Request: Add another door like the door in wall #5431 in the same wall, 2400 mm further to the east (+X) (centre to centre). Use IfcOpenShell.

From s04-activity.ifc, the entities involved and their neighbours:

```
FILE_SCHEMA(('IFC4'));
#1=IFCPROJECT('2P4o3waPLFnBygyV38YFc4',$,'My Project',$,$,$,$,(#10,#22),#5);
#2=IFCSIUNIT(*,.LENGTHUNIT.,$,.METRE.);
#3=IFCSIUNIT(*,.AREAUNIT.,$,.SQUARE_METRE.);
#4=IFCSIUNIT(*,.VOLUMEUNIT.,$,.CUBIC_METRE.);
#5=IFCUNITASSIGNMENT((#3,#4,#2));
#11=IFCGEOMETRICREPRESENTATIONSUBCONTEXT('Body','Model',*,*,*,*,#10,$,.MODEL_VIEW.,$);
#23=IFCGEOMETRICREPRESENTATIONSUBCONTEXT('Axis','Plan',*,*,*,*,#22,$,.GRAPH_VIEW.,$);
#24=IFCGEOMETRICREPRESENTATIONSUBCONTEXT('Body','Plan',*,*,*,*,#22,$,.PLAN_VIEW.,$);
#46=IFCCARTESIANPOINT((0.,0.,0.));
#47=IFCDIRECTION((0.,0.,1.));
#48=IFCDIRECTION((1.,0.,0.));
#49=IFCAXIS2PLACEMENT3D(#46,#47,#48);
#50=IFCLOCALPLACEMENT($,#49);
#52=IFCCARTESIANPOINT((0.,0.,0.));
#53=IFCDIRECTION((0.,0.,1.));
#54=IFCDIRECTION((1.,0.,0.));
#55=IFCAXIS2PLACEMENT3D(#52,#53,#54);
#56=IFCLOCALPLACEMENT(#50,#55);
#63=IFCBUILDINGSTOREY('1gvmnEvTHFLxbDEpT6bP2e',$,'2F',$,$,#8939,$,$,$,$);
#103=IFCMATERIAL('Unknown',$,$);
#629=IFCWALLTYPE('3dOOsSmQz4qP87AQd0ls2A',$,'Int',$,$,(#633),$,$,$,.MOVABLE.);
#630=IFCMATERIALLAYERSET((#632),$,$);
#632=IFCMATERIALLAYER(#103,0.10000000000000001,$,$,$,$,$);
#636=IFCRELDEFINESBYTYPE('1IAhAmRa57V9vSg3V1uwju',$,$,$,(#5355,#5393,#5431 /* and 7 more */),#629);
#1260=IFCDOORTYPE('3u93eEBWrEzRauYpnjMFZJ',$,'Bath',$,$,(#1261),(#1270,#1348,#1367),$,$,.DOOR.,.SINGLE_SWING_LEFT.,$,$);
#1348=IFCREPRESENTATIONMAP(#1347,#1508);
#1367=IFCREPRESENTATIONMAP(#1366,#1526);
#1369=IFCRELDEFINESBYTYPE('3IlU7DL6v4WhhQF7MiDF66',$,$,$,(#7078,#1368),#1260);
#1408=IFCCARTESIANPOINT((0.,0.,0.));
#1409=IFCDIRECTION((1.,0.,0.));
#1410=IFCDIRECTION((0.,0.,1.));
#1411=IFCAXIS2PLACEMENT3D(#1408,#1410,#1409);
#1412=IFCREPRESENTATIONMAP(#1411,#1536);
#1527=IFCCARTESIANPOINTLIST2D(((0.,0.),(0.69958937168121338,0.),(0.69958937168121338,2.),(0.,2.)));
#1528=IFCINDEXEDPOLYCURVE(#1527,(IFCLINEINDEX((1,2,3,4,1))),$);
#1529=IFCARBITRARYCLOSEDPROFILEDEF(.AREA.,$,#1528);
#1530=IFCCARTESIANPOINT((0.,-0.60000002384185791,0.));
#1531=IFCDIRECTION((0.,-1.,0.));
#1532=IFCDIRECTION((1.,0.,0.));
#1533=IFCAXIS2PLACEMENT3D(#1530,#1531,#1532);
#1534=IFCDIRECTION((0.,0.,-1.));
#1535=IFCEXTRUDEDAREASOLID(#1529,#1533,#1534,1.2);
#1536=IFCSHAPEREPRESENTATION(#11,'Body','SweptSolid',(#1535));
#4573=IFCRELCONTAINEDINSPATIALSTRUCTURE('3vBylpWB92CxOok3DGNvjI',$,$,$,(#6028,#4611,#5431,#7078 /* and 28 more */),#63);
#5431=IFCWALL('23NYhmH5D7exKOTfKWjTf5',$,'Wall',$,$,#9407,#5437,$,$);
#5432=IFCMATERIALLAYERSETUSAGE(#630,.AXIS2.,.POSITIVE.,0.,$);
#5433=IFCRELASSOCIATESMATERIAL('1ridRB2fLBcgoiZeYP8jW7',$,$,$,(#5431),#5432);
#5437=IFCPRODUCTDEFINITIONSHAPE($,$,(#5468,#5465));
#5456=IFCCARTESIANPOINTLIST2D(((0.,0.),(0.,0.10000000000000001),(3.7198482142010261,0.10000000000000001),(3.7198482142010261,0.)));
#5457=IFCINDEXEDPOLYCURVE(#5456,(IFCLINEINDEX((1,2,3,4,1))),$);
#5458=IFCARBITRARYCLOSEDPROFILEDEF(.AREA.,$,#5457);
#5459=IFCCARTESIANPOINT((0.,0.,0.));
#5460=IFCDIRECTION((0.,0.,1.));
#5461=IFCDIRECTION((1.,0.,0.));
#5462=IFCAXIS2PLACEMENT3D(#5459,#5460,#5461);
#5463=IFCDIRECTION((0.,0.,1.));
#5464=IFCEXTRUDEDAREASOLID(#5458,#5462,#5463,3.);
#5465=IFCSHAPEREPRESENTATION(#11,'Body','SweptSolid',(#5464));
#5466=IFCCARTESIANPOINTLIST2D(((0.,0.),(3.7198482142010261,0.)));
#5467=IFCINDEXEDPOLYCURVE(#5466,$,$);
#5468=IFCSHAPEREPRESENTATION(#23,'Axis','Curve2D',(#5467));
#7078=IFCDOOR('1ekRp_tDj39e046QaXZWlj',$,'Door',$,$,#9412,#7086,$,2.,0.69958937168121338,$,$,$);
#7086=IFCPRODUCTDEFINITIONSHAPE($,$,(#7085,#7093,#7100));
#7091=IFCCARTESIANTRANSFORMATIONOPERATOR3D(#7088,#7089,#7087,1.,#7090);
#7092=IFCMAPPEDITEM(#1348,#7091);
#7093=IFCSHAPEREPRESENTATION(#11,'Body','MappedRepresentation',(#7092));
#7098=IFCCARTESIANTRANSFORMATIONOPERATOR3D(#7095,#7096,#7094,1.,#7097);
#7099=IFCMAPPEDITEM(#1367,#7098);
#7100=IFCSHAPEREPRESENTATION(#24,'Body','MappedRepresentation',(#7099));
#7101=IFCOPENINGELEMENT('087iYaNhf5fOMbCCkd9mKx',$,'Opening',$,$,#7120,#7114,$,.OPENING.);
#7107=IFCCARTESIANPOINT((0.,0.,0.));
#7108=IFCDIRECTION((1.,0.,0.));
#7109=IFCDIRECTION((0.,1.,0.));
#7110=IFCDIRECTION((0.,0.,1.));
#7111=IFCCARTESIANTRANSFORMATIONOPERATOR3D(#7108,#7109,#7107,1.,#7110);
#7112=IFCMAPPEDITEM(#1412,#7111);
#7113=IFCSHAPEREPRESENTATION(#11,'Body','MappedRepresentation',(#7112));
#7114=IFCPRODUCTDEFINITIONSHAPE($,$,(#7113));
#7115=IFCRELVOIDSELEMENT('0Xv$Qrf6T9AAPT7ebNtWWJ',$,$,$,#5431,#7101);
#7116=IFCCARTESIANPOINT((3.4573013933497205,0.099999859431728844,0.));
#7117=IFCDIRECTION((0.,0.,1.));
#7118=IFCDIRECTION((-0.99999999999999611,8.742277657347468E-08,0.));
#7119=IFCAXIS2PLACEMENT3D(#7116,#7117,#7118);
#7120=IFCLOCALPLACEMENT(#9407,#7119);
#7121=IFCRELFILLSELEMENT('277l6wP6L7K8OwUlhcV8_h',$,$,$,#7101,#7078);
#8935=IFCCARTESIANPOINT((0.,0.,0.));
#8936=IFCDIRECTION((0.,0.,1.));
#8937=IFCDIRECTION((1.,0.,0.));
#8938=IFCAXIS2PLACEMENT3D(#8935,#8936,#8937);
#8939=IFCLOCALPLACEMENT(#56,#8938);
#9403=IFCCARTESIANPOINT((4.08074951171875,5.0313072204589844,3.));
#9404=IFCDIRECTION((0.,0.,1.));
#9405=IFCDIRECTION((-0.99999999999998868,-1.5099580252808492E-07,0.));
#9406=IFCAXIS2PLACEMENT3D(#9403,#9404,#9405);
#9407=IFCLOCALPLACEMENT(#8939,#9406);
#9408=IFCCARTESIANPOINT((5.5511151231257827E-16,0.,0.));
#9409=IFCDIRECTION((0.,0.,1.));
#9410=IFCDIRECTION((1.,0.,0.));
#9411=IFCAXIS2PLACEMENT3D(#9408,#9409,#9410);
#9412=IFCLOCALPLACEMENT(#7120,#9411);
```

```python
import ifcopenshell
import ifcopenshell.api.feature
import ifcopenshell.api.geometry
import ifcopenshell.api.root
import ifcopenshell.geom
import ifcopenshell.util.element
import ifcopenshell.util.placement
import ifcopenshell.util.shape

model = ifcopenshell.open("s04-activity.ifc")
settings = ifcopenshell.geom.settings()


def volume(element):
    """Net volume in cubic metres, openings subtracted."""
    shape = ifcopenshell.geom.create_shape(settings, element)
    return ifcopenshell.util.shape.get_volume(shape.geometry)


door = model.by_guid("1ekRp_tDj39e046QaXZWlj")
opening = door.FillsVoids[0].RelatingOpeningElement
wall = opening.VoidsElements[0].RelatingBuildingElement
before = volume(wall)
shift = ifcopenshell.util.placement.get_local_placement(wall.ObjectPlacement)[:3, 0] * -2.4

# copy_class copies the void relationship, type, container and properties, but no geometry.
new_opening = ifcopenshell.api.root.copy_class(model, product=opening)
new_opening.Representation = ifcopenshell.util.element.copy_deep(
    model, opening.Representation, exclude=["IfcGeometricRepresentationContext", "IfcRepresentationMap"]
)
new_door = ifcopenshell.api.root.copy_class(model, product=door)
new_door.Representation = ifcopenshell.util.element.copy_deep(
    model, door.Representation, exclude=["IfcGeometricRepresentationContext", "IfcRepresentationMap"]
)
ifcopenshell.api.feature.add_filling(model, opening=new_opening, element=new_door)

for old, new in ((opening, new_opening), (door, new_door)):
    matrix = ifcopenshell.util.placement.get_local_placement(old.ObjectPlacement)
    matrix[:3, 3] += shift
    ifcopenshell.api.geometry.edit_object_placement(model, product=new, matrix=matrix, is_si=False)

after = volume(wall)

print(f"wall volume {before:.3f} -> {after:.3f} m3")

model.write("s04-activity_updated.ifc")
```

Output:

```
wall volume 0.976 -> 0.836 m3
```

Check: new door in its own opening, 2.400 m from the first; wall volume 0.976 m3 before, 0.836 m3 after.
